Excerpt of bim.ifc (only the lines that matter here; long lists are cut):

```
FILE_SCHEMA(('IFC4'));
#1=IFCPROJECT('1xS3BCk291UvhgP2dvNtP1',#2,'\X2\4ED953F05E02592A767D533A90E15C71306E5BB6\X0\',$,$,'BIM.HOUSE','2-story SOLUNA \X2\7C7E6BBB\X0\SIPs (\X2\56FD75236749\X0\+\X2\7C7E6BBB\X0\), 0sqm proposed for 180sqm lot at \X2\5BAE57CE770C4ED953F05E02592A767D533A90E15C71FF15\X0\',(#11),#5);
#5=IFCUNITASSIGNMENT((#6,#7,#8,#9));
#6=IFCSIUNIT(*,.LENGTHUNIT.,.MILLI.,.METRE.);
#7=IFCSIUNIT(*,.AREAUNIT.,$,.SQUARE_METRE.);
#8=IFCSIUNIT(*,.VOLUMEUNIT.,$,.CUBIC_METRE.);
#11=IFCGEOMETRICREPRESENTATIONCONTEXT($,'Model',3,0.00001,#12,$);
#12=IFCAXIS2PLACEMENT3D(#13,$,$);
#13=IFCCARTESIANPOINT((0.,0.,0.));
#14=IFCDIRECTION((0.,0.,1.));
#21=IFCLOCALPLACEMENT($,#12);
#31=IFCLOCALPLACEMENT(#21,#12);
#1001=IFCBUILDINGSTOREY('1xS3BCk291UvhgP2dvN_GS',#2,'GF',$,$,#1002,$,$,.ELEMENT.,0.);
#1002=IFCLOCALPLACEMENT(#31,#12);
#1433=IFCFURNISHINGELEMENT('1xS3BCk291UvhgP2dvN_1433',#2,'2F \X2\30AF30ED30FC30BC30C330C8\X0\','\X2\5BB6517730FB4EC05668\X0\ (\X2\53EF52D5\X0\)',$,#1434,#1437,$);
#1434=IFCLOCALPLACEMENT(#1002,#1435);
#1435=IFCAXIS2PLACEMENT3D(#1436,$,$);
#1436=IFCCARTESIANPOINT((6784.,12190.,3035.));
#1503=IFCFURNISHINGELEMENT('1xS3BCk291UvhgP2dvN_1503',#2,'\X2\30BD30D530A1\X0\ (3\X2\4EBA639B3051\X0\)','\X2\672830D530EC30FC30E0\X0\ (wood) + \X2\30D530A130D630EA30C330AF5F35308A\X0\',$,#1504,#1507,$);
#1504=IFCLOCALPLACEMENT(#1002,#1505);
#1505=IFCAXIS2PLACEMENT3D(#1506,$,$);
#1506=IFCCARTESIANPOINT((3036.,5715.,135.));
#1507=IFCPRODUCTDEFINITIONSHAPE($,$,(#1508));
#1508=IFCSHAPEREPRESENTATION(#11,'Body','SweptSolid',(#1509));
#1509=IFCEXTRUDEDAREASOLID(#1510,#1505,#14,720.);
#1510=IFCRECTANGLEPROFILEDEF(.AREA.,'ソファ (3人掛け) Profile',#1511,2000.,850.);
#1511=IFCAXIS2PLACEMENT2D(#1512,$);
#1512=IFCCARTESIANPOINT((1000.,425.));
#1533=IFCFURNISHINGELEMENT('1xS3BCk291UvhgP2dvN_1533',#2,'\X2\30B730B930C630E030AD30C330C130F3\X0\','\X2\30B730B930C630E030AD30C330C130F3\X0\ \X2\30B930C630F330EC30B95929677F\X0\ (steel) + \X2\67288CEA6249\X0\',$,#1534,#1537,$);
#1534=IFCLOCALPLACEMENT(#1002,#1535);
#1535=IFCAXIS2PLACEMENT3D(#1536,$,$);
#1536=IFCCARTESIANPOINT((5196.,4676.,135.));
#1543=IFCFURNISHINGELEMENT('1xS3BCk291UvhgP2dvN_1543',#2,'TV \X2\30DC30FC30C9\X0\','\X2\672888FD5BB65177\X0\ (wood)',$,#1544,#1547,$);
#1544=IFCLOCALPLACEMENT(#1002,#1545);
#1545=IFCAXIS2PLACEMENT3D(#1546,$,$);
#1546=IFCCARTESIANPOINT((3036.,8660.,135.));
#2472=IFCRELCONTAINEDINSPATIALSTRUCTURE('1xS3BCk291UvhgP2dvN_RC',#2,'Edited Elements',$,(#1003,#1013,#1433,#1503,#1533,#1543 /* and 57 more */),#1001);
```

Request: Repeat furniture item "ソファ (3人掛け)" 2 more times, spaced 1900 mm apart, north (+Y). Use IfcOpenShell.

```python
import numpy as np
import ifcopenshell
import ifcopenshell.api.geometry
import ifcopenshell.api.root
import ifcopenshell.util.element
import ifcopenshell.util.placement
import ifcopenshell.util.unit

model = ifcopenshell.open("bim.ifc")
unit_scale = ifcopenshell.util.unit.calculate_unit_scale(model)


def reuse_history(source, copy):
    """copy_class also copies each property set's owner history, people and application; keep the originals."""
    for rel in copy.IsDefinedBy:
        if rel.is_a("IfcRelDefinesByProperties") and (history := rel.RelatingPropertyDefinition.OwnerHistory):
            rel.RelatingPropertyDefinition.OwnerHistory = source.OwnerHistory
            ifcopenshell.util.element.remove_deep2(model, history)


source = model.by_guid("1xS3BCk291UvhgP2dvN_1503")
base = ifcopenshell.util.placement.get_local_placement(source.ObjectPlacement)
step = np.array([0.0, 1.0, 0.0]) * 1.9 / unit_scale

for i in range(1, 3):
    copy = ifcopenshell.api.root.copy_class(model, product=source)
    copy.Representation = ifcopenshell.util.element.copy_deep(
        model, source.Representation, exclude=["IfcGeometricRepresentationContext", "IfcRepresentationMap"]
    )
    reuse_history(source, copy)
    matrix = base.copy()
    matrix[:3, 3] += i * step
    print("added at", matrix[:3, 3].round(3) + 0.0)
    ifcopenshell.api.geometry.edit_object_placement(model, product=copy, matrix=matrix, is_si=False)

model.write("bim_v2.ifc")
```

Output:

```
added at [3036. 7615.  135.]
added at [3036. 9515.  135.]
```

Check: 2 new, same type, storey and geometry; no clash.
